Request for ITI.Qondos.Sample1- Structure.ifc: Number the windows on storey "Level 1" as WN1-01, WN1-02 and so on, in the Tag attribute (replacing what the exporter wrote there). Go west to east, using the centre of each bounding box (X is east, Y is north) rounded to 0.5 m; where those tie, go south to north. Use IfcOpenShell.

First a look at what the model holds.

```python
import ifcopenshell
import ifcopenshell.util.element
import ifcopenshell.util.placement

model = ifcopenshell.open("ITI.Qondos.Sample1- Structure.ifc")
print(model.schema)
storey = next(s for s in model.by_type("IfcBuildingStorey") if s.Name == "Level 1")
windows = [e for e in ifcopenshell.util.element.get_decomposition(storey) if e.is_a("IfcWindow")]
for e in sorted(windows, key=lambda e: e.id()):
    origin = ifcopenshell.util.placement.get_local_placement(e.ObjectPlacement)[:3, 3]
    print(e.id(), e.Tag, e.Name, origin.round(2) + 0.0, sep=" | ")
```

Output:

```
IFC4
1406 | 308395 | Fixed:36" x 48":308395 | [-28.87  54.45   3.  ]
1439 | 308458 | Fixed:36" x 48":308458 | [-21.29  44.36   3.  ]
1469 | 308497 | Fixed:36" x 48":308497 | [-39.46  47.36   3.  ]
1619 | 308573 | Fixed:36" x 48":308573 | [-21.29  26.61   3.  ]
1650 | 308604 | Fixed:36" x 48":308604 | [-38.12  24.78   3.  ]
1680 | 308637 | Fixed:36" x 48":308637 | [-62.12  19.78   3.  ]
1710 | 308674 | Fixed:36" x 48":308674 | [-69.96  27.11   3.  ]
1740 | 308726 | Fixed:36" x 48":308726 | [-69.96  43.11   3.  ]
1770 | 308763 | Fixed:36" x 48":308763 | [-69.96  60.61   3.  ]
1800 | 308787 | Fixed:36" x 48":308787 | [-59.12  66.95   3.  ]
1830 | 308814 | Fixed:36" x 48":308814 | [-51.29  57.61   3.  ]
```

```python
import ifcopenshell
import ifcopenshell.geom
import ifcopenshell.util.element
import ifcopenshell.util.shape

model = ifcopenshell.open("ITI.Qondos.Sample1- Structure.ifc")
settings = ifcopenshell.geom.settings()
settings.set("use-world-coords", True)


def centre(element):
    shape = ifcopenshell.geom.create_shape(settings, element)
    return ifcopenshell.util.shape.get_bbox_centroid(shape.geometry)


storey = next(s for s in model.by_type("IfcBuildingStorey") if s.Name == "Level 1")
windows = [e for e in ifcopenshell.util.element.get_decomposition(storey) if e.is_a("IfcWindow")]

# Insertion points can sit at a corner or the storey origin, so sort by the geometry (in metres).
centres = {e: centre(e) for e in windows}
windows.sort(key=lambda e: (round(centres[e][0] / 0.5), centres[e][1]))

for i, e in enumerate(windows, start=1):
    number = f"WN1-{i:02d}"
    e.Tag = number
    print(e.id(), number)

model.write("ITI.Qondos.Sample1- Structure_edited.ifc")
```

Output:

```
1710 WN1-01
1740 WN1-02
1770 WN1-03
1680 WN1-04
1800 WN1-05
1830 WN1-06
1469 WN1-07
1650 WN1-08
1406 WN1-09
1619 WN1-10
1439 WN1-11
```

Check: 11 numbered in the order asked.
